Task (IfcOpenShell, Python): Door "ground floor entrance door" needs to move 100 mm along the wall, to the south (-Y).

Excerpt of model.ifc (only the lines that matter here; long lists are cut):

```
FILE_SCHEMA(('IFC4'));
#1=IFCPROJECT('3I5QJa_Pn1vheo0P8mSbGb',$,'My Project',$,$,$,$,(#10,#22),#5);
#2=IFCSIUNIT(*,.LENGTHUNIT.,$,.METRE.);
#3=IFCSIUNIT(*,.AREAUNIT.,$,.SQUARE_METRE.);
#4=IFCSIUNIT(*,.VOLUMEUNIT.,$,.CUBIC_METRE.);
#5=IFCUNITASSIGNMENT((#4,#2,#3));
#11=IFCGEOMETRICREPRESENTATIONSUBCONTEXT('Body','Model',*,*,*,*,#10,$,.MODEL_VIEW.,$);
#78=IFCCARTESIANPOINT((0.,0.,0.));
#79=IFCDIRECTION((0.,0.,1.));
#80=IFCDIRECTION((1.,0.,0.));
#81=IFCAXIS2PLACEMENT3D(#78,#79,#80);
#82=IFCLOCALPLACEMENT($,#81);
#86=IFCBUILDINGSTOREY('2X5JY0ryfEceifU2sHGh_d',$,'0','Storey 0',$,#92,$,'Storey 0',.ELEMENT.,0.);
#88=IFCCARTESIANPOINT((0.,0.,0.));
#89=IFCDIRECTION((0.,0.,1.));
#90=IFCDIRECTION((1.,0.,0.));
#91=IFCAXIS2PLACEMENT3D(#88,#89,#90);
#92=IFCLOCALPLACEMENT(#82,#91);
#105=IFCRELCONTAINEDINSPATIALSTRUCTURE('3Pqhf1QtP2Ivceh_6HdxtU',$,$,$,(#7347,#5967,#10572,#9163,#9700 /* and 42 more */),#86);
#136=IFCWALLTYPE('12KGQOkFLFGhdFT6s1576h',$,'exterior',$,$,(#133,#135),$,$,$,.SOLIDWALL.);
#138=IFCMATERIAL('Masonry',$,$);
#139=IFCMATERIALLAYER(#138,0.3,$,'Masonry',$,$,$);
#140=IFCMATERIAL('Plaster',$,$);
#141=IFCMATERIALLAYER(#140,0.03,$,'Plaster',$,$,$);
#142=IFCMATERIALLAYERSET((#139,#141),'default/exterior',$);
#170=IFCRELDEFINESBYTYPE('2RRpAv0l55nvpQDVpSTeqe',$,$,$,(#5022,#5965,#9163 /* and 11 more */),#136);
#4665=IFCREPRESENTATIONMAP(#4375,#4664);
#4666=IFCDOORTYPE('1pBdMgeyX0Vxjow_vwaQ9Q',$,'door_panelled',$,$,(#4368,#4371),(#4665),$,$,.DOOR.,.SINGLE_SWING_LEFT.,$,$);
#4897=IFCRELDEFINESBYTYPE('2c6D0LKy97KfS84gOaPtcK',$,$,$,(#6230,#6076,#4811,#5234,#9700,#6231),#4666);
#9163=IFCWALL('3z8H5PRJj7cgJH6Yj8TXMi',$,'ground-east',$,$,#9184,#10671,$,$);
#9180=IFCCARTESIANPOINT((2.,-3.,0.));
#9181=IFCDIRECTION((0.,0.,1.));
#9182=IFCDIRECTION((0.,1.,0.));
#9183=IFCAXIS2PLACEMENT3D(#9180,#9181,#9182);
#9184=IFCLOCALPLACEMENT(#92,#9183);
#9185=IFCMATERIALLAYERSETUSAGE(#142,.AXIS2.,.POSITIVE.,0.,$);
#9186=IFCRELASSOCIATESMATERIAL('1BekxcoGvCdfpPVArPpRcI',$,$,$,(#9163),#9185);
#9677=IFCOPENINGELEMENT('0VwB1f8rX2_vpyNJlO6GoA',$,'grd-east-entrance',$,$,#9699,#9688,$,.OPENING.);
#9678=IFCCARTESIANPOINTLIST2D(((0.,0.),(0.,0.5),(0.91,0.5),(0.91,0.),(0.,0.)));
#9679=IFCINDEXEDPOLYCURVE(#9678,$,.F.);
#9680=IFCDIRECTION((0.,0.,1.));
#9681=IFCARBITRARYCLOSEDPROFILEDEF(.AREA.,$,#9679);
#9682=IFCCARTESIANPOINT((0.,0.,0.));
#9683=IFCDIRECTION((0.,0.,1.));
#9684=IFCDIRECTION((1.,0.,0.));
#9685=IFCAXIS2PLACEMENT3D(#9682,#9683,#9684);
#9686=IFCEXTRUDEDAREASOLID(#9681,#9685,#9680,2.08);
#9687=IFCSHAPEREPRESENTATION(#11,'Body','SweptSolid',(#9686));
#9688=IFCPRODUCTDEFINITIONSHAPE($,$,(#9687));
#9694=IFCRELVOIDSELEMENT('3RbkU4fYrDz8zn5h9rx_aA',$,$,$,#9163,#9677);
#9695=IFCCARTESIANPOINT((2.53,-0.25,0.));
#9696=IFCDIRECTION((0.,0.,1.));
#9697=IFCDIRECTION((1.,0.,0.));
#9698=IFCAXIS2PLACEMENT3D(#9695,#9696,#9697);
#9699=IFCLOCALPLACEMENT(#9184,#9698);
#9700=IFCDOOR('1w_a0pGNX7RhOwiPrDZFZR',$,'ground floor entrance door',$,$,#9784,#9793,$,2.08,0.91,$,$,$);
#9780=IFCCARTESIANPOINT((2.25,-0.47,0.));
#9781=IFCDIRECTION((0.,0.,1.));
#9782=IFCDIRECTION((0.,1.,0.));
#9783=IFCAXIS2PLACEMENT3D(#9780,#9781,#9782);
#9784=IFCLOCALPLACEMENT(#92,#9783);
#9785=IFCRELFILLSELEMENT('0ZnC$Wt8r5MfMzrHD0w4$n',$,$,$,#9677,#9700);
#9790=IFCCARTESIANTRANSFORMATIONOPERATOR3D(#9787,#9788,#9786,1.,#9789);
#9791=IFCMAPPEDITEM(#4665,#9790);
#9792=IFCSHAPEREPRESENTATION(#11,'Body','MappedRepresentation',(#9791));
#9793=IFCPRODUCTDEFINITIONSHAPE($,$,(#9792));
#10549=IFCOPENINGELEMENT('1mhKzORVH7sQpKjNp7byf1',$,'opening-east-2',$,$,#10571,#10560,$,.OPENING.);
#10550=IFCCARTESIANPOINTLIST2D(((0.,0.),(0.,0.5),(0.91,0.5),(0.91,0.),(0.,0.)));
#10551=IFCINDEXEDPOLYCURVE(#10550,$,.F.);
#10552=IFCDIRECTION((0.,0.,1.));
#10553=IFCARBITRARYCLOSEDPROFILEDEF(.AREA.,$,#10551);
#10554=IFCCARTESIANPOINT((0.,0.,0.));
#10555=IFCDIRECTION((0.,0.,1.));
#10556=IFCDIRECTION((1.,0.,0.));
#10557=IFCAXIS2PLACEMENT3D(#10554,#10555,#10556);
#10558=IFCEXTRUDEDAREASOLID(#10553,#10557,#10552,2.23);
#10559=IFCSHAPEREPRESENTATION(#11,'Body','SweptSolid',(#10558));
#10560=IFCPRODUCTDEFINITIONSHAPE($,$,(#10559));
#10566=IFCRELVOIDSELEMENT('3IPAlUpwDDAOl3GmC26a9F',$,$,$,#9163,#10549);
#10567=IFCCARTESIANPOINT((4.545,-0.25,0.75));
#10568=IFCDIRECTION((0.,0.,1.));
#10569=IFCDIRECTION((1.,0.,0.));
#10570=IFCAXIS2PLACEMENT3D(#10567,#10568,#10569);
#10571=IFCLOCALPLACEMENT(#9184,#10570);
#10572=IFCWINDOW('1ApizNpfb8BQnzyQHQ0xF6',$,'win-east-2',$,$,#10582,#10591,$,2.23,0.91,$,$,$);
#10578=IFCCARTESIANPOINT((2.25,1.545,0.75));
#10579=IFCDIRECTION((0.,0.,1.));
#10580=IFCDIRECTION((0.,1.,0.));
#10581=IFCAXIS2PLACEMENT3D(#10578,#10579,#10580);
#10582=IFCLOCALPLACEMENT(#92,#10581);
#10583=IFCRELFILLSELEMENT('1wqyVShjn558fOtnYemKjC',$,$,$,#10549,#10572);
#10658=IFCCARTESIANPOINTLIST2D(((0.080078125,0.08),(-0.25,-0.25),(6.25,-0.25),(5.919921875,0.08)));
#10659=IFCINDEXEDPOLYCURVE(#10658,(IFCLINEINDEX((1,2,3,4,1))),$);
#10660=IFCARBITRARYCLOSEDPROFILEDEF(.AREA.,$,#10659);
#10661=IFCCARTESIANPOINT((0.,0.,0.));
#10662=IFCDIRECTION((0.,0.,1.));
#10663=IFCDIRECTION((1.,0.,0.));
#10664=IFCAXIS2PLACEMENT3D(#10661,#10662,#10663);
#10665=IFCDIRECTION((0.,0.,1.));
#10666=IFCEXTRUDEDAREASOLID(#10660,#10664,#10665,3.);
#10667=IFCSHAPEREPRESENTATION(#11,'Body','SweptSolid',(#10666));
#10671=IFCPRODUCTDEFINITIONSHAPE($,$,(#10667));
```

```python
import ifcopenshell
import ifcopenshell.api.geometry
import ifcopenshell.util.placement
import ifcopenshell.util.unit

model = ifcopenshell.open("model.ifc")
unit_scale = ifcopenshell.util.unit.calculate_unit_scale(model)

door = model.by_id(9700)
opening = door.FillsVoids[0].RelatingOpeningElement
wall = opening.VoidsElements[0].RelatingBuildingElement

wall_matrix = ifcopenshell.util.placement.get_local_placement(wall.ObjectPlacement)
shift = wall_matrix[:3, 0] * -0.1 / unit_scale
before = ifcopenshell.util.placement.get_local_placement(door.ObjectPlacement)[:3, 3].copy()

# The door is not placed relative to its opening, so move both.
for product in (opening, door):
    matrix = ifcopenshell.util.placement.get_local_placement(product.ObjectPlacement)
    matrix[:3, 3] += shift
    ifcopenshell.api.geometry.edit_object_placement(model, product=product, matrix=matrix, is_si=False)

after = ifcopenshell.util.placement.get_local_placement(door.ObjectPlacement)[:3, 3]
print("door moved by", (after - before).round(3) + 0.0)

model.write("model_updated.ifc")
```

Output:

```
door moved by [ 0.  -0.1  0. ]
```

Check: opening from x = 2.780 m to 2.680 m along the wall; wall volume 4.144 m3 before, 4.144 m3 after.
